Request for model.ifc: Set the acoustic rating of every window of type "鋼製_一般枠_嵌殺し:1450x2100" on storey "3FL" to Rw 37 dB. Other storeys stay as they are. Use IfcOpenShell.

First a look at what the model holds.

```python
import ifcopenshell
import ifcopenshell.util.element

model = ifcopenshell.open("model.ifc")
print(model.schema)
storey = next(s for s in model.by_type("IfcBuildingStorey") if s.Name == "3FL")
windows = [e for e in ifcopenshell.util.element.get_decomposition(storey) if e.is_a("IfcWindow")]
seen = {}
for e in windows:
    element_type = ifcopenshell.util.element.get_type(e)
    key = (element_type.Name if element_type != e and element_type else None, ifcopenshell.util.element.get_pset(e, "Pset_WindowCommon", "AcousticRating"))
    seen[key] = seen.get(key, 0) + 1
for (name, value), count in sorted(seen.items(), key=str):
    print(count, "x", name, "|", value)
```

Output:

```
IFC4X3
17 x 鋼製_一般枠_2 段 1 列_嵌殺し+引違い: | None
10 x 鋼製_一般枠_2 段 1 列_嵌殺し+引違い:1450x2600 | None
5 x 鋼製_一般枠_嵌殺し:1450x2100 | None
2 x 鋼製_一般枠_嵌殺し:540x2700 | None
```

```python
import ifcopenshell
import ifcopenshell.api.pset
import ifcopenshell.util.element

model = ifcopenshell.open("model.ifc")

storey = next(s for s in model.by_type("IfcBuildingStorey") if s.Name == "3FL")
windows = [e for e in ifcopenshell.util.element.get_decomposition(storey) if e.is_a("IfcWindow")]

count = 0
for e in windows:
    element_type = ifcopenshell.util.element.get_type(e)
    if element_type in (None, e) or element_type.Name != "鋼製_一般枠_嵌殺し:1450x2100":
        continue
    # add_pset returns the element's existing set when there is one.
    pset = ifcopenshell.api.pset.add_pset(model, product=e, name="Pset_WindowCommon")
    ifcopenshell.api.pset.edit_pset(model, pset=pset, properties={"AcousticRating": "Rw 37 dB"})
    count += 1

print(count, "windows updated")

model.write("model-out.ifc")
```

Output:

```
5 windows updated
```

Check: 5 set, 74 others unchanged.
